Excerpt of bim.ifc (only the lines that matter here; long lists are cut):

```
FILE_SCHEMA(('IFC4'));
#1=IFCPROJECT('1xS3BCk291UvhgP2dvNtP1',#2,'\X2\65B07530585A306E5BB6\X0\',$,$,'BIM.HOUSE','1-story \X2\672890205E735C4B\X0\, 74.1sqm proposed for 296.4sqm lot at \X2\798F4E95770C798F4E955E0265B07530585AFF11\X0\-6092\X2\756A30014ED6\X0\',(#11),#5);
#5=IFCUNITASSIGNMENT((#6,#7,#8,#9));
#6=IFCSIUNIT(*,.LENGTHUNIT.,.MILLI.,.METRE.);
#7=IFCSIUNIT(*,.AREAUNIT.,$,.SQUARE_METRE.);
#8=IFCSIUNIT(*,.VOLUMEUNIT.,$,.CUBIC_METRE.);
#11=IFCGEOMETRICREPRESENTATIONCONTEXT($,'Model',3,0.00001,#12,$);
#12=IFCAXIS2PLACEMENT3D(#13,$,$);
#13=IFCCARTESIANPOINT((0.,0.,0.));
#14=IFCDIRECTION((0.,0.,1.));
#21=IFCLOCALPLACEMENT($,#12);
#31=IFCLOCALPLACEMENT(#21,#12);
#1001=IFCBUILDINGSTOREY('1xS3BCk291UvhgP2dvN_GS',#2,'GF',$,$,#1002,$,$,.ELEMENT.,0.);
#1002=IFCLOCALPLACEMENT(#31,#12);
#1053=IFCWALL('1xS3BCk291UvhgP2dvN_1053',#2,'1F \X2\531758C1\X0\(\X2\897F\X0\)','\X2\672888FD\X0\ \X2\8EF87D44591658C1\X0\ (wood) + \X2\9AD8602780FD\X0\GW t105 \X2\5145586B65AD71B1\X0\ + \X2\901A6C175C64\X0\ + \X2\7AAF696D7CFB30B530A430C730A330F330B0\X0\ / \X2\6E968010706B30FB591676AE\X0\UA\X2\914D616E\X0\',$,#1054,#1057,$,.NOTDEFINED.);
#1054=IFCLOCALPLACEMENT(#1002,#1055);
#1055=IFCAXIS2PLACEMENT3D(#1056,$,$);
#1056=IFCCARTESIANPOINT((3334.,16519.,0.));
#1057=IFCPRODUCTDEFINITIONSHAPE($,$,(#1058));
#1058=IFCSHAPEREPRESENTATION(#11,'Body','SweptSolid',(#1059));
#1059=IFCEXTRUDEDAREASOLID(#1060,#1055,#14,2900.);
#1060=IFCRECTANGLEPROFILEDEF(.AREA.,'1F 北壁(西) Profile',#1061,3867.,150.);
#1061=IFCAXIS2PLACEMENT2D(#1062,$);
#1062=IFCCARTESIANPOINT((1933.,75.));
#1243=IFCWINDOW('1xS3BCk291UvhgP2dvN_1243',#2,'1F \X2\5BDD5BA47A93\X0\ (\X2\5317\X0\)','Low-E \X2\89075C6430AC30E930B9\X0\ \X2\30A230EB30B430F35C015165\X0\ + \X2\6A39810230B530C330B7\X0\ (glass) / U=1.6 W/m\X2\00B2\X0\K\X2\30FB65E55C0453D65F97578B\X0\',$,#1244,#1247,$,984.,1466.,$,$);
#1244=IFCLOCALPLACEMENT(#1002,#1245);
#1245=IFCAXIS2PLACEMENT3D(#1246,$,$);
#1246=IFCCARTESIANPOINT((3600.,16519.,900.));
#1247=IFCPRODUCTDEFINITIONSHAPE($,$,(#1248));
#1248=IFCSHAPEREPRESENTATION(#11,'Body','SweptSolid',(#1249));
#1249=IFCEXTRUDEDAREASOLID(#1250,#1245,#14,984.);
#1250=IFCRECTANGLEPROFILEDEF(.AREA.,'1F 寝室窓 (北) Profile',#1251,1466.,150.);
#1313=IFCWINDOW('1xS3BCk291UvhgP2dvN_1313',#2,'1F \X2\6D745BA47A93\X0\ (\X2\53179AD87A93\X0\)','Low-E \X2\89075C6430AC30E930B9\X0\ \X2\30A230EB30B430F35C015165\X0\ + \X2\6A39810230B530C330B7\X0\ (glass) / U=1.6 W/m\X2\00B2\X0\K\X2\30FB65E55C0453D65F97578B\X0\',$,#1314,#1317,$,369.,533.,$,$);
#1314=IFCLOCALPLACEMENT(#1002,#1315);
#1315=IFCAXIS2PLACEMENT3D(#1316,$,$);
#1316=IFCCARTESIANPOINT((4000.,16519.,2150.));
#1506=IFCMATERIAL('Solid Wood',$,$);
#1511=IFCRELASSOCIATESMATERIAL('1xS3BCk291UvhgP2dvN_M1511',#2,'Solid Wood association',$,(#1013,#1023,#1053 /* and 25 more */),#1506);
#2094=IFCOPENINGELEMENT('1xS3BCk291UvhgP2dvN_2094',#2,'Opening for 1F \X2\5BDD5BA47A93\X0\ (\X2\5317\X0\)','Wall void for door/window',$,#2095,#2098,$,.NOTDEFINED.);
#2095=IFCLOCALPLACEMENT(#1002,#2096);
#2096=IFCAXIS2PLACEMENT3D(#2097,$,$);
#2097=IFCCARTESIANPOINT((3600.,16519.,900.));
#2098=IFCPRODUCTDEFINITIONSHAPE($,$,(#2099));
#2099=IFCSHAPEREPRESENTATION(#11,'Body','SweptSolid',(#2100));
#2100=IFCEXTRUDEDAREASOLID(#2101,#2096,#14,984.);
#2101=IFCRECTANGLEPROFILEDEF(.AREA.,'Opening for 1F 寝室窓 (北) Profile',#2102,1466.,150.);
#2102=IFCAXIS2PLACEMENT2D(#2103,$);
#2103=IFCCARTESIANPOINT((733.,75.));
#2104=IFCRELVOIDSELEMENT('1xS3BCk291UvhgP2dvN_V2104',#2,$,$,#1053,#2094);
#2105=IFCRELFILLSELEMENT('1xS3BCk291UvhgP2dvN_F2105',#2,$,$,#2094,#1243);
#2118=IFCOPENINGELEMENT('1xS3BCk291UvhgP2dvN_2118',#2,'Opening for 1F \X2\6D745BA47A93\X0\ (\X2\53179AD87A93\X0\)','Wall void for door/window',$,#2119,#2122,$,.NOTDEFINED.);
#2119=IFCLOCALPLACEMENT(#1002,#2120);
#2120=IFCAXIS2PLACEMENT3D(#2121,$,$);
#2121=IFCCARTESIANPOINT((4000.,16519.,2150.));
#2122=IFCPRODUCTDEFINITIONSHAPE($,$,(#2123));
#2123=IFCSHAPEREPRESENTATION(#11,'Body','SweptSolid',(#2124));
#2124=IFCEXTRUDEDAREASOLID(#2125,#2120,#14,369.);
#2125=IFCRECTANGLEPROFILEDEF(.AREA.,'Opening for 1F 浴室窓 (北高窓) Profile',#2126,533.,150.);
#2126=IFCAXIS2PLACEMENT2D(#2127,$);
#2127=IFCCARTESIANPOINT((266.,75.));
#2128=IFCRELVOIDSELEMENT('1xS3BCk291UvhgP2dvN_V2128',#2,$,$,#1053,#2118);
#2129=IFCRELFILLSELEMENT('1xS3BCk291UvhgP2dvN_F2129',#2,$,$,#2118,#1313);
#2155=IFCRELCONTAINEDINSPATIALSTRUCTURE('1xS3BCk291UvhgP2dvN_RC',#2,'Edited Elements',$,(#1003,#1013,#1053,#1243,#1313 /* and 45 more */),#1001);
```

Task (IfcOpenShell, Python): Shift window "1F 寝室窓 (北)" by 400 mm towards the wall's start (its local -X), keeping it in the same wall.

```python
import ifcopenshell
import ifcopenshell.api.geometry
import ifcopenshell.util.placement
import ifcopenshell.util.unit

model = ifcopenshell.open("bim.ifc")
unit_scale = ifcopenshell.util.unit.calculate_unit_scale(model)

window = model.by_id(1243)
opening = window.FillsVoids[0].RelatingOpeningElement
wall = opening.VoidsElements[0].RelatingBuildingElement

wall_matrix = ifcopenshell.util.placement.get_local_placement(wall.ObjectPlacement)
shift = wall_matrix[:3, 0] * -0.4 / unit_scale
before = ifcopenshell.util.placement.get_local_placement(window.ObjectPlacement)[:3, 3].copy()

# The window is not placed relative to its opening, so move both.
for product in (opening, window):
    matrix = ifcopenshell.util.placement.get_local_placement(product.ObjectPlacement)
    matrix[:3, 3] += shift
    ifcopenshell.api.geometry.edit_object_placement(model, product=product, matrix=matrix, is_si=False)

after = ifcopenshell.util.placement.get_local_placement(window.ObjectPlacement)[:3, 3]
print("window moved by", (after - before).round(3) + 0.0)

model.write("bim_rev.ifc")
```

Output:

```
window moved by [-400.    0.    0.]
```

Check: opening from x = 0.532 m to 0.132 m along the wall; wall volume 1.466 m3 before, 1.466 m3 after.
